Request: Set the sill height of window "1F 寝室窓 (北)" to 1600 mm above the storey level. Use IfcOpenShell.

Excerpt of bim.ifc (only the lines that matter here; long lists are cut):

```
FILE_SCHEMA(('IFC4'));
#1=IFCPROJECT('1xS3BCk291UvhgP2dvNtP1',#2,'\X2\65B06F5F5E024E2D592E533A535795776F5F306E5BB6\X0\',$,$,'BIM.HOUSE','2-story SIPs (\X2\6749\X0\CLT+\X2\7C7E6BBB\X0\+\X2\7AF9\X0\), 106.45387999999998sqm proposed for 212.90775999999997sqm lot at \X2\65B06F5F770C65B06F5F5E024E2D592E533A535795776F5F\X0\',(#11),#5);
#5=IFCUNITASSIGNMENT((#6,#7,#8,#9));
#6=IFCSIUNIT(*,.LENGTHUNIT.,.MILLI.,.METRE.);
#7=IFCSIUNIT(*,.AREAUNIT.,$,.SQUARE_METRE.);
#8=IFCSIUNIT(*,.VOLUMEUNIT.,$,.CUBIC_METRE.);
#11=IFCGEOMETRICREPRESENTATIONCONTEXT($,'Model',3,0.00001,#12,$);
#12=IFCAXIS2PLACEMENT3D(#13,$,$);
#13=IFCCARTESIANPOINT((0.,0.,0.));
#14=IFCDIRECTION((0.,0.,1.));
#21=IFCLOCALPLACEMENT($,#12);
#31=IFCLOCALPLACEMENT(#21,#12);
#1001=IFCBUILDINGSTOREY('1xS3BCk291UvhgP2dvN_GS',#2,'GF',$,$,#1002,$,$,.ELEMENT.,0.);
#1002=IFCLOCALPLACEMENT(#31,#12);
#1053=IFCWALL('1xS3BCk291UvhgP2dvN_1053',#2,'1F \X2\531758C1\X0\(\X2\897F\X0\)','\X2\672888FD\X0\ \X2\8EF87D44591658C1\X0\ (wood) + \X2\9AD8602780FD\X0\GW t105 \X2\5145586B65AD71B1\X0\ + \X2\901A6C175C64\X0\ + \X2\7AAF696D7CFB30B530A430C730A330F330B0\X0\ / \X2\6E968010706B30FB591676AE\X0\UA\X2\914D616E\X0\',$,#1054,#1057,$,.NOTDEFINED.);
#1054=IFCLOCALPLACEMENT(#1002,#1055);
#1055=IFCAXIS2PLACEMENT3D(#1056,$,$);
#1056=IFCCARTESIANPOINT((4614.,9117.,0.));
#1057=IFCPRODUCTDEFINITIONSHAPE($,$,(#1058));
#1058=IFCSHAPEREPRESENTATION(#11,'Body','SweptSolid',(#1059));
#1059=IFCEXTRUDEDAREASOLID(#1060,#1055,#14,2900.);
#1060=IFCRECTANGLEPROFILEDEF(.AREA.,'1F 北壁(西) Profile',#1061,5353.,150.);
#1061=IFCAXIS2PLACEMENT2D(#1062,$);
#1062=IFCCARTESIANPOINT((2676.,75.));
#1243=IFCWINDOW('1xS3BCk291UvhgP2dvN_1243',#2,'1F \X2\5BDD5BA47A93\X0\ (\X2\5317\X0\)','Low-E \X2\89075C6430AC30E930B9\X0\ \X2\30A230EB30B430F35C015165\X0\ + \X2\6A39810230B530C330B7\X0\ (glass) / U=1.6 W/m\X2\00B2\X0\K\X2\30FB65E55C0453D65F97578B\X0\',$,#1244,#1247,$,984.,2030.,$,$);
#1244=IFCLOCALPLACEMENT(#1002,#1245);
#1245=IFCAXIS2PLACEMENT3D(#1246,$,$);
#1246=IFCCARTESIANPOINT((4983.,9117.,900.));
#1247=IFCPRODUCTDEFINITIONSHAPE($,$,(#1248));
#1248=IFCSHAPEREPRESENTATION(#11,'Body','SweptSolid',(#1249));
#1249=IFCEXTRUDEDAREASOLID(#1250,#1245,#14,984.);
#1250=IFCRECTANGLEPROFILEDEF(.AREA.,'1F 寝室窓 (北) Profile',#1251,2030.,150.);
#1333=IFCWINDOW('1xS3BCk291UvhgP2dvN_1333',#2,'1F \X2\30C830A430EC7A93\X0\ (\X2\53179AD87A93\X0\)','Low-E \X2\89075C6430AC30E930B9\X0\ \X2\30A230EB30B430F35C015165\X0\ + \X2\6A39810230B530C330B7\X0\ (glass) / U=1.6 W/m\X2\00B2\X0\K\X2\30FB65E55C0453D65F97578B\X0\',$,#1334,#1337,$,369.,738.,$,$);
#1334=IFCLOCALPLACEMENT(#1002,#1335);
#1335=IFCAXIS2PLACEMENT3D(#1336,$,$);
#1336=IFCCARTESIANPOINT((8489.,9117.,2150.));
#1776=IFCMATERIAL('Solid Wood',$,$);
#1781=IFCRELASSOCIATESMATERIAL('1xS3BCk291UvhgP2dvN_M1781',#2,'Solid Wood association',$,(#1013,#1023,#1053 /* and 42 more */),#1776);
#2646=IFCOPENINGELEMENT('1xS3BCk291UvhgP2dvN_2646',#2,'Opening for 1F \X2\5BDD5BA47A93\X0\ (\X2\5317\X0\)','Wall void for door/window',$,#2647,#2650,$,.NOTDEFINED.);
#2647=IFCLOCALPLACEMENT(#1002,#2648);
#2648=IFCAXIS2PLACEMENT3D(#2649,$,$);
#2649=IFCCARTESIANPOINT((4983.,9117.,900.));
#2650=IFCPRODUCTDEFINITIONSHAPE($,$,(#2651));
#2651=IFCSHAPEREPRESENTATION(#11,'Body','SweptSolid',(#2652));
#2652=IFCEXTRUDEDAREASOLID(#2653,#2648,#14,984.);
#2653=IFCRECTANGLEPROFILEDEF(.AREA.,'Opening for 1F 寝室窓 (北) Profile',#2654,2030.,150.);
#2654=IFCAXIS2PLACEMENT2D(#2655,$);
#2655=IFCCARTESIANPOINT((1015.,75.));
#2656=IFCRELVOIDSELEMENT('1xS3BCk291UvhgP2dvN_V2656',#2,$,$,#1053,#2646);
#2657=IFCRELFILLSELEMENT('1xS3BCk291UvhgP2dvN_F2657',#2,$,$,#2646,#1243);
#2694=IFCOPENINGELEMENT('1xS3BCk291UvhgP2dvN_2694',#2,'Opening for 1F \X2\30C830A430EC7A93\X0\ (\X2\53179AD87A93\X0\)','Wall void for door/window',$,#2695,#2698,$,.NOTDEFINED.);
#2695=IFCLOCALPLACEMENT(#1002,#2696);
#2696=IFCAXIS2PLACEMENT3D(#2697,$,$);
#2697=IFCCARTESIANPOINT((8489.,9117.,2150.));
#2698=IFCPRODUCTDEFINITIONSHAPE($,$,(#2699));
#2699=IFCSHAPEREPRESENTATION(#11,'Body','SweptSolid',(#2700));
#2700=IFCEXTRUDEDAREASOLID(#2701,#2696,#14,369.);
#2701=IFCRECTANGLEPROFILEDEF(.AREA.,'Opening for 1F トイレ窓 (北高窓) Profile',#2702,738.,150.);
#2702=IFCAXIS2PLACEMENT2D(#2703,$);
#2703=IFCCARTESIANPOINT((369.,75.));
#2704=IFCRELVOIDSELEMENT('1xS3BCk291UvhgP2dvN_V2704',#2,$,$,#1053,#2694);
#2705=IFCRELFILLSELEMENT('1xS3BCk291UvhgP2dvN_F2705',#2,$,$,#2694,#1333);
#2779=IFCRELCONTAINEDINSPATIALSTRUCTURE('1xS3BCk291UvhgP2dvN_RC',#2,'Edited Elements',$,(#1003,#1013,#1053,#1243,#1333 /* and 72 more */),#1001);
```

```python
import numpy as np
import ifcopenshell
import ifcopenshell.api.geometry
import ifcopenshell.geom
import ifcopenshell.util.element
import ifcopenshell.util.placement
import ifcopenshell.util.shape
import ifcopenshell.util.unit

model = ifcopenshell.open("bim.ifc")
unit_scale = ifcopenshell.util.unit.calculate_unit_scale(model)

window = model.by_guid("1xS3BCk291UvhgP2dvN_1243")
opening = window.FillsVoids[0].RelatingOpeningElement
storey = ifcopenshell.util.element.get_container(window, ifc_class="IfcBuildingStorey")
level = ifcopenshell.util.placement.get_local_placement(storey.ObjectPlacement)[2, 3]

# The opening's origin need not be at the sill, so measure its lowest point.
shape = ifcopenshell.geom.create_shape(ifcopenshell.geom.settings(), opening)
bottom = ifcopenshell.util.shape.get_shape_bottom_elevation(shape, shape.geometry) / unit_scale
dz = level + 1.6 / unit_scale - bottom

shift = np.array([0.0, 0.0, dz])
# The window is not placed relative to its opening, so move both.
for product in (opening, window):
    matrix = ifcopenshell.util.placement.get_local_placement(product.ObjectPlacement)
    matrix[:3, 3] += shift
    ifcopenshell.api.geometry.edit_object_placement(model, product=product, matrix=matrix, is_si=False)

print(f"moved by {dz * unit_scale:+.3f} m")

model.write("bim_rev.ifc")
```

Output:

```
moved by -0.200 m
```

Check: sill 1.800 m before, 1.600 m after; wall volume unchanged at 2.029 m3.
